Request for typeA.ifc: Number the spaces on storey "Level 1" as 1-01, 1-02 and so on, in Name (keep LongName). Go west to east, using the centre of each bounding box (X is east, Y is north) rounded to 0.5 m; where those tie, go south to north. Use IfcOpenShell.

First a look at what the model holds.

```python
import ifcopenshell
import ifcopenshell.util.element
import ifcopenshell.util.placement

model = ifcopenshell.open("typeA.ifc")
print(model.schema)
storey = next(s for s in model.by_type("IfcBuildingStorey") if s.Name == "Level 1")
spaces = [e for e in ifcopenshell.util.element.get_decomposition(storey) if e.is_a("IfcSpace")]
for e in sorted(spaces, key=lambda e: e.id()):
    origin = ifcopenshell.util.placement.get_local_placement(e.ObjectPlacement)[:3, 3]
    print(e.id(), e.Name, e.LongName, origin.round(2) + 0.0, sep=" | ")
```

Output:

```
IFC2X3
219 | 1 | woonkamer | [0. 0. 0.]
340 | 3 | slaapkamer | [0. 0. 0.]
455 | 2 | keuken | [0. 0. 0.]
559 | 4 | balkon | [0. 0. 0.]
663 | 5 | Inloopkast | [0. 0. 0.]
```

```python
import ifcopenshell
import ifcopenshell.geom
import ifcopenshell.util.element
import ifcopenshell.util.shape

model = ifcopenshell.open("typeA.ifc")
settings = ifcopenshell.geom.settings()
settings.set("use-world-coords", True)


def centre(element):
    shape = ifcopenshell.geom.create_shape(settings, element)
    return ifcopenshell.util.shape.get_bbox_centroid(shape.geometry)


storey = next(s for s in model.by_type("IfcBuildingStorey") if s.Name == "Level 1")
spaces = [e for e in ifcopenshell.util.element.get_decomposition(storey) if e.is_a("IfcSpace")]

# Insertion points can sit at a corner or the storey origin, so sort by the geometry (in metres).
centres = {e: centre(e) for e in spaces}
spaces.sort(key=lambda e: (round(centres[e][0] / 0.5), centres[e][1]))

for i, e in enumerate(spaces, start=1):
    number = f"1-{i:02d}"
    e.Name = number
    print(e.id(), number)

model.write("typeA-out.ifc")
```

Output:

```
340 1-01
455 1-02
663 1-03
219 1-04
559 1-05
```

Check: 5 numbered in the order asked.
